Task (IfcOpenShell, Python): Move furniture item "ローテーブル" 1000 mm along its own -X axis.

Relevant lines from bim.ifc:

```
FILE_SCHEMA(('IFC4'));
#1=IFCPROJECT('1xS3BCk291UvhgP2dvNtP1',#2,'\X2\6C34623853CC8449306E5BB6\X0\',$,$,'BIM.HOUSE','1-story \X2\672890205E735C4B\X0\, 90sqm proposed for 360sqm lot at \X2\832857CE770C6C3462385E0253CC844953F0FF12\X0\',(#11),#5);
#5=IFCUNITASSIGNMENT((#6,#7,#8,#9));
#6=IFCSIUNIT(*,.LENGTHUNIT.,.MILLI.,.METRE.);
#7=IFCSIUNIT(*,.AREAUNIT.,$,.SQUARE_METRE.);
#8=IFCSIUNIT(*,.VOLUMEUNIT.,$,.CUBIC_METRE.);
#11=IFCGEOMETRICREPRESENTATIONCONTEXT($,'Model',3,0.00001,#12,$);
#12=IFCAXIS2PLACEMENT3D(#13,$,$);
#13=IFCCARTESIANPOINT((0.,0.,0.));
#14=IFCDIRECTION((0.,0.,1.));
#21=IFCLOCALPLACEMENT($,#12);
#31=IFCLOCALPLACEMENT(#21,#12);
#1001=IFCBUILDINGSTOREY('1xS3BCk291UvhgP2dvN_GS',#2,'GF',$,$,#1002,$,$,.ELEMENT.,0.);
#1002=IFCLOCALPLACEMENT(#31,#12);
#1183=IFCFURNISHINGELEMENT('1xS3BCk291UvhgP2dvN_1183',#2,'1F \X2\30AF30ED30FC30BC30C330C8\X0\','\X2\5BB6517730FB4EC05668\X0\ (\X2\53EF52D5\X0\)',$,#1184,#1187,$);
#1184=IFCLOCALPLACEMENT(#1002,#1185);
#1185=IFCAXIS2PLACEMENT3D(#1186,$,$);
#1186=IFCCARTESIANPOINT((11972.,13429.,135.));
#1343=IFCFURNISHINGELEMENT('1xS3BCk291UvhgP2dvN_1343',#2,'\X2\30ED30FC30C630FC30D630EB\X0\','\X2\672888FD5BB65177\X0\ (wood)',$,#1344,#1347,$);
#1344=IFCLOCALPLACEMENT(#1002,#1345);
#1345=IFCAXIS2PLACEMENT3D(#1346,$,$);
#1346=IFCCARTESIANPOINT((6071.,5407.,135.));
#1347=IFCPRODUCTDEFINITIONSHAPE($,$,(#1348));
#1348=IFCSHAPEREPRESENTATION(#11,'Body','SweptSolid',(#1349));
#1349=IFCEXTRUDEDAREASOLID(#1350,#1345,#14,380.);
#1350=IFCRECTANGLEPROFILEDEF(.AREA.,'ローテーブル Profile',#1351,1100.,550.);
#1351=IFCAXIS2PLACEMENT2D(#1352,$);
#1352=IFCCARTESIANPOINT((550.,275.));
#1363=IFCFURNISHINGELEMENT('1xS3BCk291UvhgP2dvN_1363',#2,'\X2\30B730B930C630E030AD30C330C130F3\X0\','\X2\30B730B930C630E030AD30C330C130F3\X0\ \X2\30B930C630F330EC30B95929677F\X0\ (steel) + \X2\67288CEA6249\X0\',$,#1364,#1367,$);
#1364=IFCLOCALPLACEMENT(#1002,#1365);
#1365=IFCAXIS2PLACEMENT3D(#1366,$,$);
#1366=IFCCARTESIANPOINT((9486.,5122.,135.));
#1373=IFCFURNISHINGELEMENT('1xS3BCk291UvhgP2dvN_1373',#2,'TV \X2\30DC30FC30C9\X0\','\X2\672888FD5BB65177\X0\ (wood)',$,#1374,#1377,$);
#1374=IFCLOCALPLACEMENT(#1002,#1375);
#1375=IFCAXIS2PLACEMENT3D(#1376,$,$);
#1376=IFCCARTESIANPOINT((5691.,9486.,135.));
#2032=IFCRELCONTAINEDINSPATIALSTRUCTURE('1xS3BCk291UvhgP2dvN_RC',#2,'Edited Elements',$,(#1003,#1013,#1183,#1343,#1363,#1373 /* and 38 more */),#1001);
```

```python
import ifcopenshell
import ifcopenshell.api.geometry
import ifcopenshell.util.placement
import ifcopenshell.util.unit

model = ifcopenshell.open("bim.ifc")
unit_scale = ifcopenshell.util.unit.calculate_unit_scale(model)

item = model.by_guid("1xS3BCk291UvhgP2dvN_1343")
matrix = ifcopenshell.util.placement.get_local_placement(item.ObjectPlacement)
matrix[:3, 3] -= matrix[:3, 0] * 1 / unit_scale
ifcopenshell.api.geometry.edit_object_placement(model, product=item, matrix=matrix, is_si=False)

print(ifcopenshell.util.placement.get_local_placement(item.ObjectPlacement).round(3) + 0.0)

model.write("bim_updated.ifc")
```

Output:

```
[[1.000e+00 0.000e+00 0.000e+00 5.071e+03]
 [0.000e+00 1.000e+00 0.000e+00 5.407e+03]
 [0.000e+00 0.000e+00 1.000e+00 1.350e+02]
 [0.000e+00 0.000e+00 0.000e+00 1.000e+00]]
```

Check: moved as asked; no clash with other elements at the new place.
